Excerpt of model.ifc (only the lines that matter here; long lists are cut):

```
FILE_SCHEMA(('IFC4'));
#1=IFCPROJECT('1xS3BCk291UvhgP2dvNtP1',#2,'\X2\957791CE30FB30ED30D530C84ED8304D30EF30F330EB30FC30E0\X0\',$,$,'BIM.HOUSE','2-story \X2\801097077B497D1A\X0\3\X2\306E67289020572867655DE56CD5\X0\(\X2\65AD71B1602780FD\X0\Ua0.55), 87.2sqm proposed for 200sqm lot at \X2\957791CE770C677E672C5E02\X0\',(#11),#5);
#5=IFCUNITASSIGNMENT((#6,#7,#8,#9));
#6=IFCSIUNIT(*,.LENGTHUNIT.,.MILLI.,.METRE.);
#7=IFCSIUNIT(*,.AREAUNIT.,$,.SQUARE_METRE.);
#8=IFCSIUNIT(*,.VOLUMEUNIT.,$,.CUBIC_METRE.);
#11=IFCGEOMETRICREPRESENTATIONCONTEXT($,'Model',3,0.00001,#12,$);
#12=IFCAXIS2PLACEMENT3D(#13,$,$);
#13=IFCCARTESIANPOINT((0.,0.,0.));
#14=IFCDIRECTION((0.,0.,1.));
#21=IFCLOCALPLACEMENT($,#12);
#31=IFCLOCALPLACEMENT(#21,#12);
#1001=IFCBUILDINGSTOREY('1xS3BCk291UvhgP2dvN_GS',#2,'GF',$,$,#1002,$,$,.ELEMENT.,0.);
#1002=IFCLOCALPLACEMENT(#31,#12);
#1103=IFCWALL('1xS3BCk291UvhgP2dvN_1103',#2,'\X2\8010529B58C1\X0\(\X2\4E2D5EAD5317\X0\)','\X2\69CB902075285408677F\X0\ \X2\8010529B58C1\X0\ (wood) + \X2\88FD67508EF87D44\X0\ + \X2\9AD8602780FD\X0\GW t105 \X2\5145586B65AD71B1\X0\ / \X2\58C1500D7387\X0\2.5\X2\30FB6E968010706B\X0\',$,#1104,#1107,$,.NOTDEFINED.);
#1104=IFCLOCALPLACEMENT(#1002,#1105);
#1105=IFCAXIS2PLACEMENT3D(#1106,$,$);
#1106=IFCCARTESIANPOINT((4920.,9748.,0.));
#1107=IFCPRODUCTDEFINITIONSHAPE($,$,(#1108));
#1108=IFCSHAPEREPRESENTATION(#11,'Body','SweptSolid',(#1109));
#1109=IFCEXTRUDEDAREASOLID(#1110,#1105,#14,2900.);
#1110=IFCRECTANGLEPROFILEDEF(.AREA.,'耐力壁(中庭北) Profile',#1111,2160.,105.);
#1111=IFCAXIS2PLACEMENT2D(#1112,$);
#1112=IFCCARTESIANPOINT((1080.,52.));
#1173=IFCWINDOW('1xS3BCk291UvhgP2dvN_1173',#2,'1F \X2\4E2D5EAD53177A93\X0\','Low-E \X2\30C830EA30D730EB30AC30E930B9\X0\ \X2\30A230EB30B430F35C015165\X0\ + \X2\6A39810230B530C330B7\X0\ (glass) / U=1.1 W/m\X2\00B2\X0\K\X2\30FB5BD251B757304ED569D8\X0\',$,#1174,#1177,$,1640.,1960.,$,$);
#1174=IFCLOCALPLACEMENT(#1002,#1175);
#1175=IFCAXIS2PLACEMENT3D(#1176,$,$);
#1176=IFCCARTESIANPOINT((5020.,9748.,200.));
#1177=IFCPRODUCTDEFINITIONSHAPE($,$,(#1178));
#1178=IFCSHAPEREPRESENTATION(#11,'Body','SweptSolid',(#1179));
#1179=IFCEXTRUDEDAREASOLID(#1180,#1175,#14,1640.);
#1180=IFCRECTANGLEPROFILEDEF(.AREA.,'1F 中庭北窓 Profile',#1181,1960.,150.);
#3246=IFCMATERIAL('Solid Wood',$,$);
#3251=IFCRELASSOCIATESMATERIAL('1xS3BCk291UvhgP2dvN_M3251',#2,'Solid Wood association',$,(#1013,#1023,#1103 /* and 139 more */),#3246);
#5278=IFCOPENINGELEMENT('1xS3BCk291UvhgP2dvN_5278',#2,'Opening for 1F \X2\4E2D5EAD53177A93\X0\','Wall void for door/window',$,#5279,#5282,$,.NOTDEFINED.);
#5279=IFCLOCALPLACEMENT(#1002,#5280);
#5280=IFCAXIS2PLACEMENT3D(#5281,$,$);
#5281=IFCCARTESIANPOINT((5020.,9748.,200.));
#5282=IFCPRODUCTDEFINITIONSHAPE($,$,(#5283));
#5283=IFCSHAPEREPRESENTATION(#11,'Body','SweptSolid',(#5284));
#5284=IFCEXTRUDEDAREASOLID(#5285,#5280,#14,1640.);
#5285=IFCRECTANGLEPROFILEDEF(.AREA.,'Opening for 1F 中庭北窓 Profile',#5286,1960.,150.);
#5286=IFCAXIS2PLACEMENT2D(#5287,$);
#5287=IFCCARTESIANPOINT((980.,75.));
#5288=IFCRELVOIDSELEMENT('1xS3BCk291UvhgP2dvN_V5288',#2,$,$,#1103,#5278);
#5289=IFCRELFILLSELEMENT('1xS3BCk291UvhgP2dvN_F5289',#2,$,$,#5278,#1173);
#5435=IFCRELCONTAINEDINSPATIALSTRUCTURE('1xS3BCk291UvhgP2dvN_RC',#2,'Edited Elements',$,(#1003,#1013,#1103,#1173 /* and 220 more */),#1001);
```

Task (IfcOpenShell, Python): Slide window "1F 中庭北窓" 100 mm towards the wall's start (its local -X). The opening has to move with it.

```python
import ifcopenshell
import ifcopenshell.api.geometry
import ifcopenshell.util.placement

model = ifcopenshell.open("model.ifc")

window = model.by_id(1173)
opening = window.FillsVoids[0].RelatingOpeningElement
wall = opening.VoidsElements[0].RelatingBuildingElement

wall_matrix = ifcopenshell.util.placement.get_local_placement(wall.ObjectPlacement)
shift = wall_matrix[:3, 0] * -100.0
before = ifcopenshell.util.placement.get_local_placement(window.ObjectPlacement)[:3, 3].copy()

# The window is not placed relative to its opening, so move both.
for product in (opening, window):
    matrix = ifcopenshell.util.placement.get_local_placement(product.ObjectPlacement)
    matrix[:3, 3] += shift
    ifcopenshell.api.geometry.edit_object_placement(model, product=product, matrix=matrix, is_si=False)

after = ifcopenshell.util.placement.get_local_placement(window.ObjectPlacement)[:3, 3]
print("window moved by", (after - before).round(3) + 0.0)

model.write("model_v2.ifc")
```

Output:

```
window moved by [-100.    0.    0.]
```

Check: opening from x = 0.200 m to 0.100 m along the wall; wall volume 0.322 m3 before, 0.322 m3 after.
